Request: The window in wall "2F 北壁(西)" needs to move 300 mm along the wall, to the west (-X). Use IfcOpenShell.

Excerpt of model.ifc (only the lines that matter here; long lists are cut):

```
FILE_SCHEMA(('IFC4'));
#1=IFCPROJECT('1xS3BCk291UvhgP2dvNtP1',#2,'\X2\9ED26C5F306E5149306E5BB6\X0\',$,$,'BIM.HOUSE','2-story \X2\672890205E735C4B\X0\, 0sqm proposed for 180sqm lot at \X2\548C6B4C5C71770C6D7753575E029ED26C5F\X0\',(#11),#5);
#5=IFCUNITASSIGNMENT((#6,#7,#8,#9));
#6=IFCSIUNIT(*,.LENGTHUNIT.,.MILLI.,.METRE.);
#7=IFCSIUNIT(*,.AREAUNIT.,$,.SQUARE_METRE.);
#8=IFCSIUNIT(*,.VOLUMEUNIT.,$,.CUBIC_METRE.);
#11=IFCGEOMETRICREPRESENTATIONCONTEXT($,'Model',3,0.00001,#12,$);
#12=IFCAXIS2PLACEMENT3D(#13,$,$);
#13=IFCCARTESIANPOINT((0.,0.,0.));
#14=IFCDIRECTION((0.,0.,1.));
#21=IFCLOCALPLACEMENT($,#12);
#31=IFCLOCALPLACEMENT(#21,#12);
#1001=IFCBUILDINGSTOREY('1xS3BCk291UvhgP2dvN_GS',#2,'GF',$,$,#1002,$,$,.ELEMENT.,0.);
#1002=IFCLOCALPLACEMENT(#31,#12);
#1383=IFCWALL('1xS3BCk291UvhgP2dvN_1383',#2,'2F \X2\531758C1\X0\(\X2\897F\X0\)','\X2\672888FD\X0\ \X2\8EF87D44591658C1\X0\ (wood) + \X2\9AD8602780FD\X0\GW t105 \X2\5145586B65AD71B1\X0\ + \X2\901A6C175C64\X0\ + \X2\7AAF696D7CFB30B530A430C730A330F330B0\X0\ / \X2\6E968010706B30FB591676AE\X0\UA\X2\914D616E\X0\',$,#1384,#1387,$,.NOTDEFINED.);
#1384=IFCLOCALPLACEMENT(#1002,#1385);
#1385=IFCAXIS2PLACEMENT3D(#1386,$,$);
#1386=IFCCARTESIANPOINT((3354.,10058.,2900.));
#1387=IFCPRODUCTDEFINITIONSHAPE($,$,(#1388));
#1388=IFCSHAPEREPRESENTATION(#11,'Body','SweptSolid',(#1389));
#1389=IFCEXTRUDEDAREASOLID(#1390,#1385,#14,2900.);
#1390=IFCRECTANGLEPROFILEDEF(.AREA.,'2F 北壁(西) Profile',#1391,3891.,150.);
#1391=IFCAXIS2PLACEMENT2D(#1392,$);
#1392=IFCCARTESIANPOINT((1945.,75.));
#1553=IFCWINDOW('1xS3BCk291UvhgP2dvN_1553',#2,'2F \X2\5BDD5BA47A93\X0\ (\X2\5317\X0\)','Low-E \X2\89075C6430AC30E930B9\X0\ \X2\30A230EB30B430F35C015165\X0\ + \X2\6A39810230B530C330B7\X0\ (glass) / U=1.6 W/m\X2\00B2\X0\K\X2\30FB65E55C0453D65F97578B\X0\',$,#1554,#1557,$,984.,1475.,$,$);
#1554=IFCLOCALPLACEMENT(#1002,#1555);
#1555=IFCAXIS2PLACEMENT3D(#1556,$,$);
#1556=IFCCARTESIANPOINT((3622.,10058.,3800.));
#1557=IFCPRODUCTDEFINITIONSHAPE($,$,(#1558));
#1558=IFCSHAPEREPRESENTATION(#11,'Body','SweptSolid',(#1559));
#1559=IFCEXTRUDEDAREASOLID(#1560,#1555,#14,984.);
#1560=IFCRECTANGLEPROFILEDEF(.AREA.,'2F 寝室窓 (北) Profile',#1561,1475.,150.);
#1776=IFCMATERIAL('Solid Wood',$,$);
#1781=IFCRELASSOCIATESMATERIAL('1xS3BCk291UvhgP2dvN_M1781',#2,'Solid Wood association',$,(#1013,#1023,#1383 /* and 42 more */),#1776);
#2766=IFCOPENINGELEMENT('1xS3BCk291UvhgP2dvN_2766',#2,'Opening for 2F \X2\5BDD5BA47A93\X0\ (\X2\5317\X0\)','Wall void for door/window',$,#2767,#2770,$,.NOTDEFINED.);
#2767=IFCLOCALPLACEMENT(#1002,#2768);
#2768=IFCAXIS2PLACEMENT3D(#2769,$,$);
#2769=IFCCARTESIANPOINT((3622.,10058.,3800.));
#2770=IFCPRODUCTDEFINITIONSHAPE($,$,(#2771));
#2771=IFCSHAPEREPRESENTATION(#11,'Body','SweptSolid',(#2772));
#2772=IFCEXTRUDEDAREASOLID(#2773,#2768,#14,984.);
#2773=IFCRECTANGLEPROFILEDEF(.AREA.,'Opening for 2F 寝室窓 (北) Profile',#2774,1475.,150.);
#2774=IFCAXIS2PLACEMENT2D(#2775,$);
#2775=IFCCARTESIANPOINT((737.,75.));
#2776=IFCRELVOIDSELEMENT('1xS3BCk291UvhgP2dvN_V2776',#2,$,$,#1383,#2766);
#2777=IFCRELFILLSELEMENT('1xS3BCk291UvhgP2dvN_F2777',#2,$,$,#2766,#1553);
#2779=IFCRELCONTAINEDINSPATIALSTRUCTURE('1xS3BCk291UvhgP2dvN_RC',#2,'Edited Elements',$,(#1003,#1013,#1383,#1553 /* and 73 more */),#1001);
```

```python
import ifcopenshell
import ifcopenshell.api.geometry
import ifcopenshell.util.placement
import ifcopenshell.util.unit

model = ifcopenshell.open("model.ifc")
unit_scale = ifcopenshell.util.unit.calculate_unit_scale(model)

window = model.by_guid("1xS3BCk291UvhgP2dvN_1553")
opening = window.FillsVoids[0].RelatingOpeningElement
wall = opening.VoidsElements[0].RelatingBuildingElement

wall_matrix = ifcopenshell.util.placement.get_local_placement(wall.ObjectPlacement)
shift = wall_matrix[:3, 0] * -0.3 / unit_scale
before = ifcopenshell.util.placement.get_local_placement(window.ObjectPlacement)[:3, 3].copy()

# The window is not placed relative to its opening, so move both.
for product in (opening, window):
    matrix = ifcopenshell.util.placement.get_local_placement(product.ObjectPlacement)
    matrix[:3, 3] += shift
    ifcopenshell.api.geometry.edit_object_placement(model, product=product, matrix=matrix, is_si=False)

after = ifcopenshell.util.placement.get_local_placement(window.ObjectPlacement)[:3, 3]
print("window moved by", (after - before).round(3) + 0.0)

model.write("model_v2.ifc")
```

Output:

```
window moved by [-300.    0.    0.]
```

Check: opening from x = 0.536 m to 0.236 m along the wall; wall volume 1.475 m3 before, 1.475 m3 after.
